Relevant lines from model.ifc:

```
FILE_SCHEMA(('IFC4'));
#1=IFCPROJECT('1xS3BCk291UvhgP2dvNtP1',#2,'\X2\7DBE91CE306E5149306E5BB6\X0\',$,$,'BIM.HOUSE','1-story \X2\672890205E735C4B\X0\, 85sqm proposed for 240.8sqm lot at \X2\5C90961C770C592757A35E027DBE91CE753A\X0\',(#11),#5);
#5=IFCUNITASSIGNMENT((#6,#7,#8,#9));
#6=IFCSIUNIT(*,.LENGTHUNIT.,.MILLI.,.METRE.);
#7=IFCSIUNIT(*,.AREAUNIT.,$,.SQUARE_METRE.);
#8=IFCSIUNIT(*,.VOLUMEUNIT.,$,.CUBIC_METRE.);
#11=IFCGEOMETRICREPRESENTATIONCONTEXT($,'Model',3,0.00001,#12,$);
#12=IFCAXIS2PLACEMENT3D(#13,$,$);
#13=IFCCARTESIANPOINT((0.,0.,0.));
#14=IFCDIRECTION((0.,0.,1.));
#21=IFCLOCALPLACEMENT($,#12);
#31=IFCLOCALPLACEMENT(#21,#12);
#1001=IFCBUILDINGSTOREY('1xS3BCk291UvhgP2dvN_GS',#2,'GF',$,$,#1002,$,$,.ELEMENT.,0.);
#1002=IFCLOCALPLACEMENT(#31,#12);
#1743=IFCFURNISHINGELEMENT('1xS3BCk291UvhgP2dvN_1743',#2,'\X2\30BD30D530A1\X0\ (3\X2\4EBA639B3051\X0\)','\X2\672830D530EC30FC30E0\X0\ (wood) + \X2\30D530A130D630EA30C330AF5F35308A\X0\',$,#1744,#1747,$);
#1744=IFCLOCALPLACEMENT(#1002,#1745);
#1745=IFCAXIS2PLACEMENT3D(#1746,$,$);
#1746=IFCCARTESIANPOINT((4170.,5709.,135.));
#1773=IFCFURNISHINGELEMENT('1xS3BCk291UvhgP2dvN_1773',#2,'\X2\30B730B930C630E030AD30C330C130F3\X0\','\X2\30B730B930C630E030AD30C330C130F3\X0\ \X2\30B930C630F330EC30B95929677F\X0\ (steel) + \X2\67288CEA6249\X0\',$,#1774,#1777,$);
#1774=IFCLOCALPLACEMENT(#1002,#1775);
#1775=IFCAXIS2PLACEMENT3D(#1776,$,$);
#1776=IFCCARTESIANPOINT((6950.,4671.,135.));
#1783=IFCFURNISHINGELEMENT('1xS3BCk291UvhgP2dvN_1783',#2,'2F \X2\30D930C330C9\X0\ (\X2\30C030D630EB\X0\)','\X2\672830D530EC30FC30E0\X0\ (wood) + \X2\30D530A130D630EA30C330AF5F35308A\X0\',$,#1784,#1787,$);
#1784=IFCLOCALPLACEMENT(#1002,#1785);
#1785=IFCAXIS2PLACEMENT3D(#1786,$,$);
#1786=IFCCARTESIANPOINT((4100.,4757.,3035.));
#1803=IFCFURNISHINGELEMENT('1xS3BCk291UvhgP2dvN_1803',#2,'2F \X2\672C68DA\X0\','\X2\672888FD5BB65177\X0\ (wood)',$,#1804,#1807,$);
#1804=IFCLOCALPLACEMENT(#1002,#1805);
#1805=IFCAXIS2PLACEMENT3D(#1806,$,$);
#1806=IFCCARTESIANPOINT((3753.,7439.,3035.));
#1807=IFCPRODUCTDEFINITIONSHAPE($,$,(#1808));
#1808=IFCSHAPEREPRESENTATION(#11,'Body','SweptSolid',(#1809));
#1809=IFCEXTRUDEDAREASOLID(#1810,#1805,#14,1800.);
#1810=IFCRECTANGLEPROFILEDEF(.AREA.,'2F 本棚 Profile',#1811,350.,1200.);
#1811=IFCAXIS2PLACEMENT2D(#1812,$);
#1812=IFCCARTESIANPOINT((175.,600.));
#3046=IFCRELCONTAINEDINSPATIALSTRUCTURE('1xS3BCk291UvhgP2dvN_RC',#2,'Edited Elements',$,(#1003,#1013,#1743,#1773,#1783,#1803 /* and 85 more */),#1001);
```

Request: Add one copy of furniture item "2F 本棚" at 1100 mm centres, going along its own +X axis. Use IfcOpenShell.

```python
import ifcopenshell
import ifcopenshell.api.geometry
import ifcopenshell.api.root
import ifcopenshell.util.element
import ifcopenshell.util.placement
import ifcopenshell.util.unit

model = ifcopenshell.open("model.ifc")
unit_scale = ifcopenshell.util.unit.calculate_unit_scale(model)


def reuse_history(source, copy):
    """copy_class also copies each property set's owner history, people and application; keep the originals."""
    for rel in copy.IsDefinedBy:
        if rel.is_a("IfcRelDefinesByProperties") and (history := rel.RelatingPropertyDefinition.OwnerHistory):
            rel.RelatingPropertyDefinition.OwnerHistory = source.OwnerHistory
            ifcopenshell.util.element.remove_deep2(model, history)


source = model.by_guid("1xS3BCk291UvhgP2dvN_1803")
base = ifcopenshell.util.placement.get_local_placement(source.ObjectPlacement)
step = base[:3, 0] * 1.1 / unit_scale

for i in range(1, 2):
    copy = ifcopenshell.api.root.copy_class(model, product=source)
    copy.Representation = ifcopenshell.util.element.copy_deep(
        model, source.Representation, exclude=["IfcGeometricRepresentationContext", "IfcRepresentationMap"]
    )
    reuse_history(source, copy)
    matrix = base.copy()
    matrix[:3, 3] += i * step
    print("added at", matrix[:3, 3].round(3) + 0.0)
    ifcopenshell.api.geometry.edit_object_placement(model, product=copy, matrix=matrix, is_si=False)

model.write("model-out.ifc")
```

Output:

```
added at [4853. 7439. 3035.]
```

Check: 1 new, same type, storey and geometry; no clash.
